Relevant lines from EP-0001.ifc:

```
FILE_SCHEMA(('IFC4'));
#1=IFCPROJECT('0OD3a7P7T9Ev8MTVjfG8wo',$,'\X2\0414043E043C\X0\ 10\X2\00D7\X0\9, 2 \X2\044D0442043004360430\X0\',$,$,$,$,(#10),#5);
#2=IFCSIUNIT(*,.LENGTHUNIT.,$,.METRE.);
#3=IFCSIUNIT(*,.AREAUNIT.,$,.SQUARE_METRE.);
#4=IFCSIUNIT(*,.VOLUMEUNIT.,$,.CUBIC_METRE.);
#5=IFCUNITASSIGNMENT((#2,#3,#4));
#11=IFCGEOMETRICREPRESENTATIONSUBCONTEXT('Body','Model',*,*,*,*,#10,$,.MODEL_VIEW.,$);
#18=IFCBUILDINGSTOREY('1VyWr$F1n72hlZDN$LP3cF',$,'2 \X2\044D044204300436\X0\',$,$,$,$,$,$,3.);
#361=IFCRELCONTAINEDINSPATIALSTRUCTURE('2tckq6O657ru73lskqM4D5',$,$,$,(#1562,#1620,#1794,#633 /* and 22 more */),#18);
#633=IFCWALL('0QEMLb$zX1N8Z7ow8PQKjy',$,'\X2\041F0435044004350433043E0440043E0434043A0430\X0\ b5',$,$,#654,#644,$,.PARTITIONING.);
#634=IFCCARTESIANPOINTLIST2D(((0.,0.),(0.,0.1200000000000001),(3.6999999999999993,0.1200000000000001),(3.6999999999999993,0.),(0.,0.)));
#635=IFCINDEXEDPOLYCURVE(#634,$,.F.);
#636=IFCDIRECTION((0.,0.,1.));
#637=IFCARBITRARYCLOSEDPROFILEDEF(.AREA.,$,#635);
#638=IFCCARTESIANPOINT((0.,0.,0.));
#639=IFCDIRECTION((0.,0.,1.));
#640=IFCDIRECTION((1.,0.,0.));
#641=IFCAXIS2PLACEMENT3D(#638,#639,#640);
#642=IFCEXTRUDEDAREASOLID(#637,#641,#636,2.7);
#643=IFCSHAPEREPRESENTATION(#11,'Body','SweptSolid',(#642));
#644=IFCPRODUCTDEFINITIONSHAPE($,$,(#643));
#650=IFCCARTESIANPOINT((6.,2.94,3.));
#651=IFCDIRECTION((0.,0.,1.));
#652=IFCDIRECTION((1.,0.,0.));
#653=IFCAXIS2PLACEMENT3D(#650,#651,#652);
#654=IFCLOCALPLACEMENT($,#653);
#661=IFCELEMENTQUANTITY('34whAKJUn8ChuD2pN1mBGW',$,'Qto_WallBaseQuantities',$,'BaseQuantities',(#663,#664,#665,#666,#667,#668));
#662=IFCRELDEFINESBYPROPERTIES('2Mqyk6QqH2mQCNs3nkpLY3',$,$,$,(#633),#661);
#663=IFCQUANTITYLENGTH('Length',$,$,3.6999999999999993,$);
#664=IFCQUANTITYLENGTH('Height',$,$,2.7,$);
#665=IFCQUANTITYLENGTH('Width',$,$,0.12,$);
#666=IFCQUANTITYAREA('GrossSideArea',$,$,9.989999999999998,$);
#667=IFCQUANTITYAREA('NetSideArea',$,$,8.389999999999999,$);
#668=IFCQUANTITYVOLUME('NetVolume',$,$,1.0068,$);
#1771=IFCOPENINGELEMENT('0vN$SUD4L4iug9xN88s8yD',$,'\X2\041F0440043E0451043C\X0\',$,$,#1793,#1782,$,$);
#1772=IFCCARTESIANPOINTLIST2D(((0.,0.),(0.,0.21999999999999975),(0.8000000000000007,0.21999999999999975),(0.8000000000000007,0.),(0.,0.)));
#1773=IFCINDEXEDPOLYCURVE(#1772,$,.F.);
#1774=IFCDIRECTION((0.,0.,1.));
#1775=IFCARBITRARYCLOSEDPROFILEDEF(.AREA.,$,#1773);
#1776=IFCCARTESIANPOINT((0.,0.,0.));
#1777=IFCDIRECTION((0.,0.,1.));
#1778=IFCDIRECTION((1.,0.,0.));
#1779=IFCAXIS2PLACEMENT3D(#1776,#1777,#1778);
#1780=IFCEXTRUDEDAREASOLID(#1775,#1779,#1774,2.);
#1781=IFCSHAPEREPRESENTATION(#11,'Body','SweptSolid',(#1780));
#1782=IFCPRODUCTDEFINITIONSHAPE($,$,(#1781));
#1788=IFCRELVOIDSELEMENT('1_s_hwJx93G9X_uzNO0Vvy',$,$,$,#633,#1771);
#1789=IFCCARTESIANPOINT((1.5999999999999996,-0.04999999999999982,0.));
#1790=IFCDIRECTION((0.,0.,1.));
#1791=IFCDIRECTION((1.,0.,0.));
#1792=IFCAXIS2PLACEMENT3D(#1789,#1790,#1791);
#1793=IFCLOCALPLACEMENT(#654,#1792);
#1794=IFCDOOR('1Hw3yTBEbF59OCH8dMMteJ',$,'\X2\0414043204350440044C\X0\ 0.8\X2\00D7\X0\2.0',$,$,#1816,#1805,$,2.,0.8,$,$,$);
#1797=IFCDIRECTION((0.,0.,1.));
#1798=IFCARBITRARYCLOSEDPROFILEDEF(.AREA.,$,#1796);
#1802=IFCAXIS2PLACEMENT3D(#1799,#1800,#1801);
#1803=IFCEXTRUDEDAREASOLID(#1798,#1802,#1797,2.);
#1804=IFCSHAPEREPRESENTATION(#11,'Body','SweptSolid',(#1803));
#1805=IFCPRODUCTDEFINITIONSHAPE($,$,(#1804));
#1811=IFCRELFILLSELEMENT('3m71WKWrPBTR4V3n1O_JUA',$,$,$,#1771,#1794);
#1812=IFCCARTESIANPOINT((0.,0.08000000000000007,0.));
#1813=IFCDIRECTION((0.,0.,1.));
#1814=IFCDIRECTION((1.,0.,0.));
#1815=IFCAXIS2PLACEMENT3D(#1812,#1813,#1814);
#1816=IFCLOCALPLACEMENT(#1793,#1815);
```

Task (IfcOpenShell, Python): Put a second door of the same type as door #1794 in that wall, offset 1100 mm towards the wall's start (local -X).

```python
import ifcopenshell
import ifcopenshell.api.feature
import ifcopenshell.api.geometry
import ifcopenshell.api.pset
import ifcopenshell.api.root
import ifcopenshell.geom
import ifcopenshell.util.element
import ifcopenshell.util.placement
import ifcopenshell.util.shape
import ifcopenshell.util.unit

model = ifcopenshell.open("EP-0001.ifc")
unit_scale = ifcopenshell.util.unit.calculate_unit_scale(model)
area_scale = ifcopenshell.util.unit.calculate_unit_scale(model, "AREAUNIT")
volume_scale = ifcopenshell.util.unit.calculate_unit_scale(model, "VOLUMEUNIT")
settings = ifcopenshell.geom.settings()


def volume(element):
    """Net volume in cubic metres, openings subtracted."""
    shape = ifcopenshell.geom.create_shape(settings, element)
    return ifcopenshell.util.shape.get_volume(shape.geometry)


door = model.by_guid("1Hw3yTBEbF59OCH8dMMteJ")
opening = door.FillsVoids[0].RelatingOpeningElement
wall = opening.VoidsElements[0].RelatingBuildingElement
before = volume(wall)
shift = ifcopenshell.util.placement.get_local_placement(wall.ObjectPlacement)[:3, 0] * -1.1 / unit_scale

# copy_class copies the void relationship, type, container and properties, but no geometry.
new_opening = ifcopenshell.api.root.copy_class(model, product=opening)
new_opening.Representation = ifcopenshell.util.element.copy_deep(
    model, opening.Representation, exclude=["IfcGeometricRepresentationContext", "IfcRepresentationMap"]
)
new_door = ifcopenshell.api.root.copy_class(model, product=door)
new_door.Representation = ifcopenshell.util.element.copy_deep(
    model, door.Representation, exclude=["IfcGeometricRepresentationContext", "IfcRepresentationMap"]
)
ifcopenshell.api.feature.add_filling(model, opening=new_opening, element=new_door)

for old, new in ((opening, new_opening), (door, new_door)):
    matrix = ifcopenshell.util.placement.get_local_placement(old.ObjectPlacement)
    matrix[:3, 3] += shift
    ifcopenshell.api.geometry.edit_object_placement(model, product=new, matrix=matrix, is_si=False)

after = volume(wall)
thickness = 0.12  # wall thickness in metres

# Update the wall's stored quantities.
qto = model.by_id(ifcopenshell.util.element.get_pset(wall, "Qto_WallBaseQuantities", should_inherit=False)["id"])
ifcopenshell.api.pset.edit_qto(model, qto=qto, properties={
    "NetSideArea": after / thickness / area_scale,
    "NetVolume": after / volume_scale,
})

print(f"wall volume {before:.3f} -> {after:.3f} m3")

model.write("EP-0001_rev.ifc")
```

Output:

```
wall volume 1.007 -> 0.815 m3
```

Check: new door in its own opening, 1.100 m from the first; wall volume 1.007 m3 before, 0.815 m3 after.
